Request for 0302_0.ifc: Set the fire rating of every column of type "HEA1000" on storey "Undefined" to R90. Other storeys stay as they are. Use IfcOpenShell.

First a look at what the model holds.

```python
import ifcopenshell
import ifcopenshell.util.element

model = ifcopenshell.open("0302_0.ifc")
print(model.schema)
storey = next(s for s in model.by_type("IfcBuildingStorey") if s.Name == "Undefined")
columns = [e for e in ifcopenshell.util.element.get_decomposition(storey) if e.is_a("IfcColumn")]
seen = {}
for e in columns:
    element_type = ifcopenshell.util.element.get_type(e)
    key = (element_type.Name if element_type != e and element_type else None, ifcopenshell.util.element.get_pset(e, "Pset_ColumnCommon", "FireRating"))
    seen[key] = seen.get(key, 0) + 1
for (name, value), count in sorted(seen.items(), key=str):
    print(count, "x", name, "|", value)
```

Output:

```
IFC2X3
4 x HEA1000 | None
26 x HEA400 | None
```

```python
import ifcopenshell
import ifcopenshell.api.pset
import ifcopenshell.util.element

model = ifcopenshell.open("0302_0.ifc")

storey = next(s for s in model.by_type("IfcBuildingStorey") if s.Name == "Undefined")
columns = [e for e in ifcopenshell.util.element.get_decomposition(storey) if e.is_a("IfcColumn")]

count = 0
for e in columns:
    element_type = ifcopenshell.util.element.get_type(e)
    if element_type in (None, e) or element_type.Name != "HEA1000":
        continue
    found = ifcopenshell.util.element.get_pset(e, "Pset_ColumnCommon", should_inherit=False)
    if found:
        pset = model.by_id(found["id"])
        if len(ifcopenshell.util.element.get_elements_by_pset(pset)) > 1:
            pset = ifcopenshell.api.pset.unshare_pset(model, products=[e], pset=pset)[0]
    else:
        pset = ifcopenshell.api.pset.add_pset(model, product=e, name="Pset_ColumnCommon")
    ifcopenshell.api.pset.edit_pset(model, pset=pset, properties={"FireRating": "R90"})
    count += 1

print(count, "columns updated")

model.write("0302_0_rev.ifc")
```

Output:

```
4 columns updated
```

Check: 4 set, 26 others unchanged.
